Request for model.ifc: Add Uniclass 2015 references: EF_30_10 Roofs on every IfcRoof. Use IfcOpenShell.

First a look at what the model holds.

```python
import ifcopenshell

model = ifcopenshell.open("model.ifc")
print(model.schema)
print("classifications:", [c.Name for c in model.by_type("IfcClassification")])
for ifc_class in ("IfcDoor", "IfcRoof", "IfcStair", "IfcWall", "IfcWindow"):
    print(ifc_class, len(model.by_type(ifc_class)))
```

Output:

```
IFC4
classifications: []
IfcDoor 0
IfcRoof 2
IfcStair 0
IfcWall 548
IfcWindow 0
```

```python
import ifcopenshell
import ifcopenshell.api.classification

model = ifcopenshell.open("model.ifc")

system = ifcopenshell.api.classification.add_classification(model, classification="Uniclass 2015")

codes = {
    "IfcRoof": ("EF_30_10", "Roofs"),
}
for ifc_class, (code, name) in codes.items():
    products = model.by_type(ifc_class)
    ifcopenshell.api.classification.add_reference(
        model, products=products, classification=system, identification=code, name=name
    )
    print(code, len(products))

model.write("model_rev.ifc")
```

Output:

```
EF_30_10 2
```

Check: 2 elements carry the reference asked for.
